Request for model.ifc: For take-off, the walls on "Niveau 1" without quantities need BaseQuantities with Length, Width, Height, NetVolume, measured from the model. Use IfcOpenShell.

First a look at what the model holds.

```python
import ifcopenshell
import ifcopenshell.util.element
import ifcopenshell.util.unit

model = ifcopenshell.open("model.ifc")
print(model.schema)
for unit_type in ("LENGTHUNIT", "AREAUNIT", "VOLUMEUNIT"):
    print(unit_type, ifcopenshell.util.unit.calculate_unit_scale(model, unit_type))
storey = next(s for s in model.by_type("IfcBuildingStorey") if s.Name == "Niveau 1")
walls = [e for e in ifcopenshell.util.element.get_decomposition(storey) if e.is_a("IfcWall")]
for e in sorted(walls, key=lambda e: e.id()):
    print(e.id(), e.is_a(), e.Name, list(ifcopenshell.util.element.get_psets(e, qtos_only=True)), sep=" | ")
```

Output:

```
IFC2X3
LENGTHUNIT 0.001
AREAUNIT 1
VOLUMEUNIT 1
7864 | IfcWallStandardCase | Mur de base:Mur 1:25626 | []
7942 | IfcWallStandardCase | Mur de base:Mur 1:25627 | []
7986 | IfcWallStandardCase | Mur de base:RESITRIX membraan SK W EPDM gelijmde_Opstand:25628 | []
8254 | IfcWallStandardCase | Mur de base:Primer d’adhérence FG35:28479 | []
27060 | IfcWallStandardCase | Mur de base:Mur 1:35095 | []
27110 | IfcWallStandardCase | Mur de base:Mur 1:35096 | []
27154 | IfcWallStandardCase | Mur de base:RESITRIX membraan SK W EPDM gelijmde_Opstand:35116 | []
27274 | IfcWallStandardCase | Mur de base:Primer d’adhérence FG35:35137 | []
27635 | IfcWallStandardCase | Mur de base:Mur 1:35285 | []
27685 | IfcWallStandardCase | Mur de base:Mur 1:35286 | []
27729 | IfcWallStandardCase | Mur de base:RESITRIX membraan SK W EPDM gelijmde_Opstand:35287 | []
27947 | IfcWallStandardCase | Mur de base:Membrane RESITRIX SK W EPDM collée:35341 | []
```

```python
import ifcopenshell
import ifcopenshell.api.pset
import ifcopenshell.geom
import ifcopenshell.util.element
import ifcopenshell.util.shape
import ifcopenshell.util.unit

model = ifcopenshell.open("model.ifc")
unit_scale = ifcopenshell.util.unit.calculate_unit_scale(model)
volume_scale = ifcopenshell.util.unit.calculate_unit_scale(model, "VOLUMEUNIT")
settings = ifcopenshell.geom.settings()

storey = next(s for s in model.by_type("IfcBuildingStorey") if s.Name == "Niveau 1")
walls = [e for e in ifcopenshell.util.element.get_decomposition(storey) if e.is_a("IfcWall")]

for e in sorted(walls, key=lambda e: e.id()):
    if ifcopenshell.util.element.get_psets(e, qtos_only=True, should_inherit=False):
        continue
    # Geometry comes back in metres, in the element's own axes.
    shape = ifcopenshell.geom.create_shape(settings, e)
    values = {
        "Length": ifcopenshell.util.shape.get_x(shape.geometry) / unit_scale,
        "Width": ifcopenshell.util.shape.get_y(shape.geometry) / unit_scale,
        "Height": ifcopenshell.util.shape.get_z(shape.geometry) / unit_scale,
        "NetVolume": ifcopenshell.util.shape.get_volume(shape.geometry) / volume_scale,
    }
    qto = ifcopenshell.api.pset.add_qto(model, product=e, name="BaseQuantities")
    ifcopenshell.api.pset.edit_qto(model, qto=qto, properties=values)
    print(e.id(), {k: round(v, 3) for k, v in values.items()})

model.write("model_updated.ifc")
```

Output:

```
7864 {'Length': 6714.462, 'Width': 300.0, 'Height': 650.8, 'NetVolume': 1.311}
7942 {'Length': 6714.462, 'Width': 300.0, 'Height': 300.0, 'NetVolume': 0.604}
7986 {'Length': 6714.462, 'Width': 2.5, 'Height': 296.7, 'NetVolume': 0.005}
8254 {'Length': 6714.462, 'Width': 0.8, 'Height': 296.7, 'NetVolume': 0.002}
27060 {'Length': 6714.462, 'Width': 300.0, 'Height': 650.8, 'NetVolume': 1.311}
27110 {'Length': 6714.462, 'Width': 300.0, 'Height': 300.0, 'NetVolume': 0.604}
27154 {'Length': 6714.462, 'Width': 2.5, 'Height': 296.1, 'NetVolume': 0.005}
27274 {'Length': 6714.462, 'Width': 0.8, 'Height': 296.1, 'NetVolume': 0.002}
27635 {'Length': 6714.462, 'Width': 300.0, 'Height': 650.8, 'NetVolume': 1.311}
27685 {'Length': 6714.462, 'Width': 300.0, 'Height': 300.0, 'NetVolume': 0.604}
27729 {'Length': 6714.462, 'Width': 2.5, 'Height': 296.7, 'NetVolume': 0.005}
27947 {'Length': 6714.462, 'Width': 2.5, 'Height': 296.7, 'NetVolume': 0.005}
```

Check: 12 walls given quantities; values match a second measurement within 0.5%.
